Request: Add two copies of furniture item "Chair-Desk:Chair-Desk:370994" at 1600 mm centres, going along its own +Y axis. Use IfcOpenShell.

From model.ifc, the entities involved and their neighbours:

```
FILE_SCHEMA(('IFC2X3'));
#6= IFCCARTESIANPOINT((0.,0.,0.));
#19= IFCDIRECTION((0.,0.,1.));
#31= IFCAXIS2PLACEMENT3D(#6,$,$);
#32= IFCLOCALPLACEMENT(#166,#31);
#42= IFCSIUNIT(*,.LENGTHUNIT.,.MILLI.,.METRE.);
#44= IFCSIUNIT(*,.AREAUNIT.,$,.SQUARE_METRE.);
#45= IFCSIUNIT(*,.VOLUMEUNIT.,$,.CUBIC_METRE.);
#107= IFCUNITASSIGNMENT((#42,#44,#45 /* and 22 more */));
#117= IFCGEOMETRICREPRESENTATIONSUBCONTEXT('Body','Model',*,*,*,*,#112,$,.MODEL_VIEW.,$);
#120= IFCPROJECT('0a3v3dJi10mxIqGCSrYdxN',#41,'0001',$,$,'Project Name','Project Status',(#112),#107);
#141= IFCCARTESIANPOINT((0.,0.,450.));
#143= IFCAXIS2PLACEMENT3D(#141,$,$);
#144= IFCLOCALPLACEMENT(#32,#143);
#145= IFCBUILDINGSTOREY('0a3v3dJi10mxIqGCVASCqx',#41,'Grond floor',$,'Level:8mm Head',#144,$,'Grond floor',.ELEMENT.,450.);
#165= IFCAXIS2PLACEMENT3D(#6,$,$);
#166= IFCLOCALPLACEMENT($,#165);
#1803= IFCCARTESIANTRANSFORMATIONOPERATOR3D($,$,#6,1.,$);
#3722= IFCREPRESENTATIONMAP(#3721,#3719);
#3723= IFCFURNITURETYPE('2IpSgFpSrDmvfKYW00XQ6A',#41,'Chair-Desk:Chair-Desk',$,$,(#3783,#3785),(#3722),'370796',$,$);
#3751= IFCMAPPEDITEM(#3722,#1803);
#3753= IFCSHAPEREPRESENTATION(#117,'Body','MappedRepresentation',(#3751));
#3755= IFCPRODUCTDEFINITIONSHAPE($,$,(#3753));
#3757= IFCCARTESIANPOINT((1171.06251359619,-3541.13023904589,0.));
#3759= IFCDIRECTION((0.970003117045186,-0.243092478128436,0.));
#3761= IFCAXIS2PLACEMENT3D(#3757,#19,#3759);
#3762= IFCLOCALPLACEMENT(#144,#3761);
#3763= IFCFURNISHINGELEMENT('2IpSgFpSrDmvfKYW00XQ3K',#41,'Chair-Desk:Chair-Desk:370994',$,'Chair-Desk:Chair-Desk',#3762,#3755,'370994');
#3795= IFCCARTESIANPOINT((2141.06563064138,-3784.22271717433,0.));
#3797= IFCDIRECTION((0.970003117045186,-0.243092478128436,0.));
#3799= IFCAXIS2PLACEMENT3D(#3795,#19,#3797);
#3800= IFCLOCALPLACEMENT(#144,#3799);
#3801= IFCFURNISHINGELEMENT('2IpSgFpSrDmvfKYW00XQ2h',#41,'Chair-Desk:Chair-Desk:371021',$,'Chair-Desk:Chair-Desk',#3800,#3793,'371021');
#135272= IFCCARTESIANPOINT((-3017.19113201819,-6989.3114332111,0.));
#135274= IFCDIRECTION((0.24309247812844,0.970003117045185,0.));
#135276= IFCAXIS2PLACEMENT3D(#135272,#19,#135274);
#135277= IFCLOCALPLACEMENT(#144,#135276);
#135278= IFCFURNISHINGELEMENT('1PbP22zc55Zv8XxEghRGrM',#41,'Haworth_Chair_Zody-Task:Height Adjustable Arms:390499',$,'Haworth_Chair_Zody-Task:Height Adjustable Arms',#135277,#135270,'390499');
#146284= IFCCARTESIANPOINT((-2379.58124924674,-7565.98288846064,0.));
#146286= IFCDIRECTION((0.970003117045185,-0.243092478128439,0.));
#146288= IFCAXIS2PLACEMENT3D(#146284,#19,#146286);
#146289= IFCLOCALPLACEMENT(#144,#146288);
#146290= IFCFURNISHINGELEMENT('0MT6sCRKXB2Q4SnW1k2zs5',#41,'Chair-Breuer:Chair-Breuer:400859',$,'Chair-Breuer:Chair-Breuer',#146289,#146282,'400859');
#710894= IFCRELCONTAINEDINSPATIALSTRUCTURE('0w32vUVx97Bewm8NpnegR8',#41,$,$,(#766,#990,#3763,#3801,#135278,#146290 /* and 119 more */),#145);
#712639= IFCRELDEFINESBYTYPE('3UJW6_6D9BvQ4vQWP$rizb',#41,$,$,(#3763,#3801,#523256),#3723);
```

```python
import ifcopenshell
import ifcopenshell.api.geometry
import ifcopenshell.api.root
import ifcopenshell.util.element
import ifcopenshell.util.placement

model = ifcopenshell.open("model.ifc")


def reuse_history(source, copy):
    """copy_class also copies each property set's owner history, people and application; keep the originals."""
    for rel in copy.IsDefinedBy:
        if rel.is_a("IfcRelDefinesByProperties") and (history := rel.RelatingPropertyDefinition.OwnerHistory):
            rel.RelatingPropertyDefinition.OwnerHistory = source.OwnerHistory
            ifcopenshell.util.element.remove_deep2(model, history)


source = model.by_id(3763)
base = ifcopenshell.util.placement.get_local_placement(source.ObjectPlacement)
step = base[:3, 1] * 1600.0

for i in range(1, 3):
    copy = ifcopenshell.api.root.copy_class(model, product=source)
    copy.Representation = ifcopenshell.util.element.copy_deep(
        model, source.Representation, exclude=["IfcGeometricRepresentationContext", "IfcRepresentationMap"]
    )
    copy.Name = "Chair-Desk:Chair-Desk"
    copy.Tag = None
    reuse_history(source, copy)
    matrix = base.copy()
    matrix[:3, 3] += i * step
    print("added at", matrix[:3, 3].round(3) + 0.0)
    ifcopenshell.api.geometry.edit_object_placement(model, product=copy, matrix=matrix, is_si=False)

model.write("model-out.ifc")
```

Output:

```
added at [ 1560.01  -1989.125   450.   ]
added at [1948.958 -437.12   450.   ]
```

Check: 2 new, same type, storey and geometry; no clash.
